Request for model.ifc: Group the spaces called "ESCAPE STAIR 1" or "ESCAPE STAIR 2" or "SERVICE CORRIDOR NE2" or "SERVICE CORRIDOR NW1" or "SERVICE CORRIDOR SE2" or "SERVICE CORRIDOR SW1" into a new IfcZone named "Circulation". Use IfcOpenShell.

First a look at what the model holds.

```python
import ifcopenshell

model = ifcopenshell.open("model.ifc")
print(model.schema)
seen = {}
for space in model.by_type("IfcSpace"):
    seen[space.LongName] = seen.get(space.LongName, 0) + 1
for name, count in sorted(seen.items(), key=str):
    print(count, "x", name)
print("zones:", [z.Name for z in model.by_type("IfcZone")][:20])
```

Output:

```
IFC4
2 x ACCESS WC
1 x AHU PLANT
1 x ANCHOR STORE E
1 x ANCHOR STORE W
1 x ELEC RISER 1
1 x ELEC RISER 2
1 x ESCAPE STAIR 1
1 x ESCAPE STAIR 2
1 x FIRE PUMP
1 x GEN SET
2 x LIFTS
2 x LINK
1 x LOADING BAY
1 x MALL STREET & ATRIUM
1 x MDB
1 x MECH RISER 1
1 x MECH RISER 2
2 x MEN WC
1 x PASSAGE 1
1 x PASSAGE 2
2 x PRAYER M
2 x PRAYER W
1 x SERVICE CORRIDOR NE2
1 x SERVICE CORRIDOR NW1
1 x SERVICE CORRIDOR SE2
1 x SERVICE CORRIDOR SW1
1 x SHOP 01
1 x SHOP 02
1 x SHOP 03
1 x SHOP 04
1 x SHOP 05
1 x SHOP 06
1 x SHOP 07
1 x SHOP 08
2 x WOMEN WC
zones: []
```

```python
import ifcopenshell
import ifcopenshell.api.group
import ifcopenshell.api.root

model = ifcopenshell.open("model.ifc")

names = {"ESCAPE STAIR 1", "ESCAPE STAIR 2", "SERVICE CORRIDOR NE2", "SERVICE CORRIDOR NW1", "SERVICE CORRIDOR SE2", "SERVICE CORRIDOR SW1"}
spaces = [s for s in model.by_type("IfcSpace") if s.LongName in names]

zone = ifcopenshell.api.root.create_entity(model, ifc_class="IfcZone", name="Circulation")
ifcopenshell.api.group.assign_group(model, products=spaces, group=zone)
print(len(spaces), "spaces in", zone.Name)

model.write("model_rev.ifc")
```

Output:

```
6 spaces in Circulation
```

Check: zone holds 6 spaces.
